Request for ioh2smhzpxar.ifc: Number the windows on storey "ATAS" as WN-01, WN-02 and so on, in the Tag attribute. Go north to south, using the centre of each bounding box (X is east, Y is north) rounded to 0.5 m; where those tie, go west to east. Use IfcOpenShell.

First a look at what the model holds.

```python
import ifcopenshell
import ifcopenshell.util.element
import ifcopenshell.util.placement

model = ifcopenshell.open("ioh2smhzpxar.ifc")
print(model.schema)
storey = next(s for s in model.by_type("IfcBuildingStorey") if s.Name == "ATAS")
windows = [e for e in ifcopenshell.util.element.get_decomposition(storey) if e.is_a("IfcWindow")]
for e in sorted(windows, key=lambda e: e.id()):
    origin = ifcopenshell.util.placement.get_local_placement(e.ObjectPlacement)[:3, 3]
    print(e.id(), e.Tag, e.Name, origin.round(2) + 0.0, sep=" | ")
```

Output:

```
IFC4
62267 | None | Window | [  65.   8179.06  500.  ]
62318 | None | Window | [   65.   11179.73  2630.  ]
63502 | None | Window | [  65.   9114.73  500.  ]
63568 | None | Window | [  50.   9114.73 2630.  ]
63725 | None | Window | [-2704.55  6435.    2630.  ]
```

```python
import ifcopenshell
import ifcopenshell.geom
import ifcopenshell.util.element
import ifcopenshell.util.shape

model = ifcopenshell.open("ioh2smhzpxar.ifc")
settings = ifcopenshell.geom.settings()
settings.set("use-world-coords", True)


def centre(element):
    shape = ifcopenshell.geom.create_shape(settings, element)
    return ifcopenshell.util.shape.get_bbox_centroid(shape.geometry)


storey = next(s for s in model.by_type("IfcBuildingStorey") if s.Name == "ATAS")
windows = [e for e in ifcopenshell.util.element.get_decomposition(storey) if e.is_a("IfcWindow")]

# Insertion points can sit at a corner or the storey origin, so sort by the geometry (in metres).
centres = {e: centre(e) for e in windows}
windows.sort(key=lambda e: (-round(centres[e][1] / 0.5), centres[e][0]))

for i, e in enumerate(windows, start=1):
    number = f"WN-{i:02d}"
    e.Tag = number
    print(e.id(), number)

model.write("ioh2smhzpxar_v2.ifc")
```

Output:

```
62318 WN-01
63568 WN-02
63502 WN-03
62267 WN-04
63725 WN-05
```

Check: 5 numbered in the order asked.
